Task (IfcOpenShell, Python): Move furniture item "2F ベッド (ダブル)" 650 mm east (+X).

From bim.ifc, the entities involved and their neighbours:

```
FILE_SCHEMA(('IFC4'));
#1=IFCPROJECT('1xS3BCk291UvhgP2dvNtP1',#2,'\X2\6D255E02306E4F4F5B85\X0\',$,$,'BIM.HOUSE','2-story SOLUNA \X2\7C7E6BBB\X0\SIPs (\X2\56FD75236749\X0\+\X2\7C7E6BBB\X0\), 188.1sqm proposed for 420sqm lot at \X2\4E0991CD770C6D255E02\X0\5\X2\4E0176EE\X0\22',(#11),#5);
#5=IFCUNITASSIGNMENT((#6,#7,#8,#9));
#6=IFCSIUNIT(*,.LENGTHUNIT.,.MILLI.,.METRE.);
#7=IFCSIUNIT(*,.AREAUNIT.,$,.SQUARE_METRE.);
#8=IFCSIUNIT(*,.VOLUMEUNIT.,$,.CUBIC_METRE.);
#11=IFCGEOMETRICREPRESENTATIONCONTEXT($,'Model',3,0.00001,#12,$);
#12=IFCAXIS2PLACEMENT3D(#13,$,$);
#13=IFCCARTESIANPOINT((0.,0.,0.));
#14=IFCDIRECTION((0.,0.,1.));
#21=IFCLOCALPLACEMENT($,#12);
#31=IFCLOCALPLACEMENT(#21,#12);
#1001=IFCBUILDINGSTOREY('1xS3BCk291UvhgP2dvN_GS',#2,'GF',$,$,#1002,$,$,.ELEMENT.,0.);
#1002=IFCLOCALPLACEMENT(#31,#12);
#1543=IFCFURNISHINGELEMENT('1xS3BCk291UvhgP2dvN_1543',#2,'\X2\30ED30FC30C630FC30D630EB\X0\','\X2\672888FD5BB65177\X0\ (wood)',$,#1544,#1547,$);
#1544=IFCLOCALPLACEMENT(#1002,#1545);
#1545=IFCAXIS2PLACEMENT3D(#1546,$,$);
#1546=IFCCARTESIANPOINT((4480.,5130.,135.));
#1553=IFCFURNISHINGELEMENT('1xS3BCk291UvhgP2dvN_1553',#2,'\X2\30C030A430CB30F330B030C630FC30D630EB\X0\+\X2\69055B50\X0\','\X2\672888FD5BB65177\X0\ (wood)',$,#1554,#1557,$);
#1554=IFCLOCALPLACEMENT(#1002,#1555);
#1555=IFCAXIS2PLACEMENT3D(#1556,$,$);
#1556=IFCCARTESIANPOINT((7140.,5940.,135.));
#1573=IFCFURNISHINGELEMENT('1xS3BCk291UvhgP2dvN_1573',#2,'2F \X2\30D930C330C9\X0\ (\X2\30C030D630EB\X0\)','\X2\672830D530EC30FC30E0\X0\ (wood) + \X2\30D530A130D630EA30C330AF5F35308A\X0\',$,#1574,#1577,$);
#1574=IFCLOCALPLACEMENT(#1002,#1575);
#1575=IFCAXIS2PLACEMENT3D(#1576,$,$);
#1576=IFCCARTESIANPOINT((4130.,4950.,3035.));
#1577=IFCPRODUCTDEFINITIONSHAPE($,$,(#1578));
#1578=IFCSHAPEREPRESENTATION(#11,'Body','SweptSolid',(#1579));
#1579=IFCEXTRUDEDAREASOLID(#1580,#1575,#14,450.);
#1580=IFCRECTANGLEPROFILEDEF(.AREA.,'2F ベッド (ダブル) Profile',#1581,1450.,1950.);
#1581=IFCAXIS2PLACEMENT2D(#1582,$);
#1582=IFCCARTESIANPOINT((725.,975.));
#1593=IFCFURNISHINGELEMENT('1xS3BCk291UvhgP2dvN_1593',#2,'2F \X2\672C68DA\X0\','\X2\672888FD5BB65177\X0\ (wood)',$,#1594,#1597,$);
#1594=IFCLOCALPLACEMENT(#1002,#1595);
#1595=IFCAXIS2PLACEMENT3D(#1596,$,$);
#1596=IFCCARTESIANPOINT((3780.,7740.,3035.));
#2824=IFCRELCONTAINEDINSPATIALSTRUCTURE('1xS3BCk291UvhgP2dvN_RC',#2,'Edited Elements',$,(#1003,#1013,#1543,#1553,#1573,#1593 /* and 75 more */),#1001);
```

```python
import ifcopenshell
import ifcopenshell.api.geometry
import ifcopenshell.util.placement

model = ifcopenshell.open("bim.ifc")

item = model.by_guid("1xS3BCk291UvhgP2dvN_1573")
matrix = ifcopenshell.util.placement.get_local_placement(item.ObjectPlacement)
matrix[0, 3] += 650.0
ifcopenshell.api.geometry.edit_object_placement(model, product=item, matrix=matrix, is_si=False)

print(ifcopenshell.util.placement.get_local_placement(item.ObjectPlacement).round(3) + 0.0)

model.write("bim_edited.ifc")
```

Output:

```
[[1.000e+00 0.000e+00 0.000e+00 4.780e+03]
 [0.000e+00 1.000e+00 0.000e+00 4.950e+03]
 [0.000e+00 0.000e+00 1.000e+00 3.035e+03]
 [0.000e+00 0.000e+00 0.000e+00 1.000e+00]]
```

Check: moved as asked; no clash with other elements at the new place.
